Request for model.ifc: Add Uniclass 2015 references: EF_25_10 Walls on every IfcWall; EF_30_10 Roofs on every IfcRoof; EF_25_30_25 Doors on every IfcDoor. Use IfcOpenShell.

First a look at what the model holds.

```python
import ifcopenshell

model = ifcopenshell.open("model.ifc")
print(model.schema)
print("classifications:", [c.Name for c in model.by_type("IfcClassification")])
for ifc_class in ("IfcDoor", "IfcRoof", "IfcStair", "IfcWall", "IfcWindow"):
    print(ifc_class, len(model.by_type(ifc_class)))
```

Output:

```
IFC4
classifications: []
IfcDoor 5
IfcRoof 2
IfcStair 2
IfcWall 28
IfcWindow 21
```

```python
import ifcopenshell
import ifcopenshell.api.classification

model = ifcopenshell.open("model.ifc")

system = ifcopenshell.api.classification.add_classification(model, classification="Uniclass 2015")

codes = {
    "IfcWall": ("EF_25_10", "Walls"),
    "IfcRoof": ("EF_30_10", "Roofs"),
    "IfcDoor": ("EF_25_30_25", "Doors"),
}
for ifc_class, (code, name) in codes.items():
    products = model.by_type(ifc_class)
    ifcopenshell.api.classification.add_reference(
        model, products=products, classification=system, identification=code, name=name
    )
    print(code, len(products))

model.write("model_updated.ifc")
```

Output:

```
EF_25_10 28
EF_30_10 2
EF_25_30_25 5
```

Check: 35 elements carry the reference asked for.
